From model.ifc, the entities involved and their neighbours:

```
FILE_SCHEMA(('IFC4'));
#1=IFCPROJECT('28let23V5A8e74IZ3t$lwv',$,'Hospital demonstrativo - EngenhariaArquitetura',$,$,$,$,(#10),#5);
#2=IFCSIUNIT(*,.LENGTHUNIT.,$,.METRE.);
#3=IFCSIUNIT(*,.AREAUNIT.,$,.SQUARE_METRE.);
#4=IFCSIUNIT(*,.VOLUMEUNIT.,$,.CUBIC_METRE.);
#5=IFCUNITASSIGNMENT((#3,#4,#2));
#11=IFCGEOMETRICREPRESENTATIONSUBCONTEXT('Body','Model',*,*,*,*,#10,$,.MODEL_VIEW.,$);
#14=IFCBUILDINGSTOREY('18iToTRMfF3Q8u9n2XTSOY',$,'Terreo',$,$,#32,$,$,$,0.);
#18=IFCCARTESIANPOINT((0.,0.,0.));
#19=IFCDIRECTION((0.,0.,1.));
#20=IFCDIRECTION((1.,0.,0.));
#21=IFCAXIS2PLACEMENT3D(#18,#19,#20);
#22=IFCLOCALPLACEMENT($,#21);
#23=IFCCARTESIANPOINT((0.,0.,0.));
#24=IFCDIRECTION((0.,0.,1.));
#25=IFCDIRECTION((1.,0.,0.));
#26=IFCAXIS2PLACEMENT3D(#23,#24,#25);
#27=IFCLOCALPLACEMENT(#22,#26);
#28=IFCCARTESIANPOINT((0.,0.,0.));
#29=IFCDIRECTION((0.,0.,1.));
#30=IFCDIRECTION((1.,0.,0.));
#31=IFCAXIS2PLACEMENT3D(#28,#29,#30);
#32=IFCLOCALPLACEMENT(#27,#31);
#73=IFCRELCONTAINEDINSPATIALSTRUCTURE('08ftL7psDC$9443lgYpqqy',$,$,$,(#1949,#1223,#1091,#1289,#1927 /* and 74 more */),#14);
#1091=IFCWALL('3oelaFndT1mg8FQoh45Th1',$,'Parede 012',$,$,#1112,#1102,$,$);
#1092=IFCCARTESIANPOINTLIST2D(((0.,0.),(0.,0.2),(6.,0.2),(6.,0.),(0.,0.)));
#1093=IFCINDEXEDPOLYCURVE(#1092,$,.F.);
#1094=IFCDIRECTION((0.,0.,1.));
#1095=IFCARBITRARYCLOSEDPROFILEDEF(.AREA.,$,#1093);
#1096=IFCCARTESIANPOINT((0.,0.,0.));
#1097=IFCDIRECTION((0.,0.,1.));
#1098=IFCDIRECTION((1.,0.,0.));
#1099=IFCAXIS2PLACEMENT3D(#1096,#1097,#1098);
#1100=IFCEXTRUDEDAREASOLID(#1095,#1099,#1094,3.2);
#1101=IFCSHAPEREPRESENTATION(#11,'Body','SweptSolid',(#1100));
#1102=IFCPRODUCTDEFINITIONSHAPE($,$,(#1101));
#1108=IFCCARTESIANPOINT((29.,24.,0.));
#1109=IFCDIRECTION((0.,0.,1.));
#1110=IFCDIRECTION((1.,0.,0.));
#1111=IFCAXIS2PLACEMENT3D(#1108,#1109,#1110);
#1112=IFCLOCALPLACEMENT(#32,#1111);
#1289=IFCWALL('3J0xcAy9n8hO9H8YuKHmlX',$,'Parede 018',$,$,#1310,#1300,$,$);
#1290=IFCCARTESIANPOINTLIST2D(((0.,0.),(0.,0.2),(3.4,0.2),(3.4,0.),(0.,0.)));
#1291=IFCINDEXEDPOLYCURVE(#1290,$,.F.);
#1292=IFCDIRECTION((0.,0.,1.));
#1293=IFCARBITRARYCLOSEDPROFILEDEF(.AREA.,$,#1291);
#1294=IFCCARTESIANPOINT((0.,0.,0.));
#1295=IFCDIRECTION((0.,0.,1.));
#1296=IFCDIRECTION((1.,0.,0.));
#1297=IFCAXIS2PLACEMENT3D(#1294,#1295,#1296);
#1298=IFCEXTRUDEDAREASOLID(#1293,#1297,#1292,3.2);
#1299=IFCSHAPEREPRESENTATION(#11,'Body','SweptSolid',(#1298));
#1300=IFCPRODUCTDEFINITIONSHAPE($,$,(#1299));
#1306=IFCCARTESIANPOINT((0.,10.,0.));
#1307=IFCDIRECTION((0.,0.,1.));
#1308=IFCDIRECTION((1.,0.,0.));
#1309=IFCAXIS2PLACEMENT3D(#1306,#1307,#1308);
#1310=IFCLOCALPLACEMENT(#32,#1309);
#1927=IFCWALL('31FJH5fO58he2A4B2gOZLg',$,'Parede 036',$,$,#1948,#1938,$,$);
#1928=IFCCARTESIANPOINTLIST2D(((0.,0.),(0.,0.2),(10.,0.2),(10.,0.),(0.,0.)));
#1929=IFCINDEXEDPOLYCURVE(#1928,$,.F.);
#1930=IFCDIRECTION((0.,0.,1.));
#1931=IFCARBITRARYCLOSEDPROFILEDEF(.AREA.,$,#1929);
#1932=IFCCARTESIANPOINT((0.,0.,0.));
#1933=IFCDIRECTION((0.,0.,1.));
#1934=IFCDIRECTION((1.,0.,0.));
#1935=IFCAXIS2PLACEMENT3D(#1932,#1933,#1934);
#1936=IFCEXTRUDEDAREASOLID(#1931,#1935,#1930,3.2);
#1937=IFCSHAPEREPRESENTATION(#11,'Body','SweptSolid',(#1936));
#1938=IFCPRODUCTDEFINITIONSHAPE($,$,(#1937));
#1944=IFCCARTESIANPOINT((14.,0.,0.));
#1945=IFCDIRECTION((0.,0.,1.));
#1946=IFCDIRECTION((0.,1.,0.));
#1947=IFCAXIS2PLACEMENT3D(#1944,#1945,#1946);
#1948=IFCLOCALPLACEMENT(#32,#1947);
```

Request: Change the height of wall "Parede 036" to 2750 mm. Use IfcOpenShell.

```python
import ifcopenshell
import ifcopenshell.geom
import ifcopenshell.util.representation
import ifcopenshell.util.shape
import ifcopenshell.util.unit

model = ifcopenshell.open("model.ifc")
unit_scale = ifcopenshell.util.unit.calculate_unit_scale(model)
settings = ifcopenshell.geom.settings()


def volume(element):
    """Net volume in cubic metres, openings subtracted."""
    shape = ifcopenshell.geom.create_shape(settings, element)
    return ifcopenshell.util.shape.get_volume(shape.geometry)


wall = model.by_guid("31FJH5fO58he2A4B2gOZLg")
before = volume(wall)

body = ifcopenshell.util.representation.get_representation(wall, "Model", "Body")
solid = body.Items[0]
old_height = solid.Depth
solid.Depth = 2.75 / unit_scale
after = volume(wall)

print(f"height {old_height:g} -> {solid.Depth:g}, volume {before:.3f} -> {after:.3f} m3")

model.write("model_rev.ifc")
```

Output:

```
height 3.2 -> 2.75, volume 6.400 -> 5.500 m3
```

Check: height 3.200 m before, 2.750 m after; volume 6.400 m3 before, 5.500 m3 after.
